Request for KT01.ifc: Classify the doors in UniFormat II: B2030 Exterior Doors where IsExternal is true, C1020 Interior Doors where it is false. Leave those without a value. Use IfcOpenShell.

First a look at what the model holds.

```python
import ifcopenshell
import ifcopenshell.util.element

model = ifcopenshell.open("KT01.ifc")
print(model.schema)
print("classifications:", [c.Name for c in model.by_type("IfcClassification")])
values = [ifcopenshell.util.element.get_pset(e, "Pset_DoorCommon", "IsExternal") for e in model.by_type("IfcDoor")]
for value in (True, False, None):
    print("IsExternal", value, values.count(value))
```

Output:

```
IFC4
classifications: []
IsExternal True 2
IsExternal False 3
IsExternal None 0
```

```python
import ifcopenshell
import ifcopenshell.api.classification
import ifcopenshell.util.element

model = ifcopenshell.open("KT01.ifc")

system = ifcopenshell.api.classification.add_classification(model, classification="UniFormat II")

doors = model.by_type("IfcDoor")
external = {e: ifcopenshell.util.element.get_pset(e, "Pset_DoorCommon", "IsExternal") for e in doors}
for flag, code, name in ((True, "B2030", "Exterior Doors"), (False, "C1020", "Interior Doors")):
    products = [e for e in doors if external[e] is flag]
    ifcopenshell.api.classification.add_reference(
        model, products=products, classification=system, identification=code, name=name
    )
    print(code, len(products))

model.write("KT01_v2.ifc")
```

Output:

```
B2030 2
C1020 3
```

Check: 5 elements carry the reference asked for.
